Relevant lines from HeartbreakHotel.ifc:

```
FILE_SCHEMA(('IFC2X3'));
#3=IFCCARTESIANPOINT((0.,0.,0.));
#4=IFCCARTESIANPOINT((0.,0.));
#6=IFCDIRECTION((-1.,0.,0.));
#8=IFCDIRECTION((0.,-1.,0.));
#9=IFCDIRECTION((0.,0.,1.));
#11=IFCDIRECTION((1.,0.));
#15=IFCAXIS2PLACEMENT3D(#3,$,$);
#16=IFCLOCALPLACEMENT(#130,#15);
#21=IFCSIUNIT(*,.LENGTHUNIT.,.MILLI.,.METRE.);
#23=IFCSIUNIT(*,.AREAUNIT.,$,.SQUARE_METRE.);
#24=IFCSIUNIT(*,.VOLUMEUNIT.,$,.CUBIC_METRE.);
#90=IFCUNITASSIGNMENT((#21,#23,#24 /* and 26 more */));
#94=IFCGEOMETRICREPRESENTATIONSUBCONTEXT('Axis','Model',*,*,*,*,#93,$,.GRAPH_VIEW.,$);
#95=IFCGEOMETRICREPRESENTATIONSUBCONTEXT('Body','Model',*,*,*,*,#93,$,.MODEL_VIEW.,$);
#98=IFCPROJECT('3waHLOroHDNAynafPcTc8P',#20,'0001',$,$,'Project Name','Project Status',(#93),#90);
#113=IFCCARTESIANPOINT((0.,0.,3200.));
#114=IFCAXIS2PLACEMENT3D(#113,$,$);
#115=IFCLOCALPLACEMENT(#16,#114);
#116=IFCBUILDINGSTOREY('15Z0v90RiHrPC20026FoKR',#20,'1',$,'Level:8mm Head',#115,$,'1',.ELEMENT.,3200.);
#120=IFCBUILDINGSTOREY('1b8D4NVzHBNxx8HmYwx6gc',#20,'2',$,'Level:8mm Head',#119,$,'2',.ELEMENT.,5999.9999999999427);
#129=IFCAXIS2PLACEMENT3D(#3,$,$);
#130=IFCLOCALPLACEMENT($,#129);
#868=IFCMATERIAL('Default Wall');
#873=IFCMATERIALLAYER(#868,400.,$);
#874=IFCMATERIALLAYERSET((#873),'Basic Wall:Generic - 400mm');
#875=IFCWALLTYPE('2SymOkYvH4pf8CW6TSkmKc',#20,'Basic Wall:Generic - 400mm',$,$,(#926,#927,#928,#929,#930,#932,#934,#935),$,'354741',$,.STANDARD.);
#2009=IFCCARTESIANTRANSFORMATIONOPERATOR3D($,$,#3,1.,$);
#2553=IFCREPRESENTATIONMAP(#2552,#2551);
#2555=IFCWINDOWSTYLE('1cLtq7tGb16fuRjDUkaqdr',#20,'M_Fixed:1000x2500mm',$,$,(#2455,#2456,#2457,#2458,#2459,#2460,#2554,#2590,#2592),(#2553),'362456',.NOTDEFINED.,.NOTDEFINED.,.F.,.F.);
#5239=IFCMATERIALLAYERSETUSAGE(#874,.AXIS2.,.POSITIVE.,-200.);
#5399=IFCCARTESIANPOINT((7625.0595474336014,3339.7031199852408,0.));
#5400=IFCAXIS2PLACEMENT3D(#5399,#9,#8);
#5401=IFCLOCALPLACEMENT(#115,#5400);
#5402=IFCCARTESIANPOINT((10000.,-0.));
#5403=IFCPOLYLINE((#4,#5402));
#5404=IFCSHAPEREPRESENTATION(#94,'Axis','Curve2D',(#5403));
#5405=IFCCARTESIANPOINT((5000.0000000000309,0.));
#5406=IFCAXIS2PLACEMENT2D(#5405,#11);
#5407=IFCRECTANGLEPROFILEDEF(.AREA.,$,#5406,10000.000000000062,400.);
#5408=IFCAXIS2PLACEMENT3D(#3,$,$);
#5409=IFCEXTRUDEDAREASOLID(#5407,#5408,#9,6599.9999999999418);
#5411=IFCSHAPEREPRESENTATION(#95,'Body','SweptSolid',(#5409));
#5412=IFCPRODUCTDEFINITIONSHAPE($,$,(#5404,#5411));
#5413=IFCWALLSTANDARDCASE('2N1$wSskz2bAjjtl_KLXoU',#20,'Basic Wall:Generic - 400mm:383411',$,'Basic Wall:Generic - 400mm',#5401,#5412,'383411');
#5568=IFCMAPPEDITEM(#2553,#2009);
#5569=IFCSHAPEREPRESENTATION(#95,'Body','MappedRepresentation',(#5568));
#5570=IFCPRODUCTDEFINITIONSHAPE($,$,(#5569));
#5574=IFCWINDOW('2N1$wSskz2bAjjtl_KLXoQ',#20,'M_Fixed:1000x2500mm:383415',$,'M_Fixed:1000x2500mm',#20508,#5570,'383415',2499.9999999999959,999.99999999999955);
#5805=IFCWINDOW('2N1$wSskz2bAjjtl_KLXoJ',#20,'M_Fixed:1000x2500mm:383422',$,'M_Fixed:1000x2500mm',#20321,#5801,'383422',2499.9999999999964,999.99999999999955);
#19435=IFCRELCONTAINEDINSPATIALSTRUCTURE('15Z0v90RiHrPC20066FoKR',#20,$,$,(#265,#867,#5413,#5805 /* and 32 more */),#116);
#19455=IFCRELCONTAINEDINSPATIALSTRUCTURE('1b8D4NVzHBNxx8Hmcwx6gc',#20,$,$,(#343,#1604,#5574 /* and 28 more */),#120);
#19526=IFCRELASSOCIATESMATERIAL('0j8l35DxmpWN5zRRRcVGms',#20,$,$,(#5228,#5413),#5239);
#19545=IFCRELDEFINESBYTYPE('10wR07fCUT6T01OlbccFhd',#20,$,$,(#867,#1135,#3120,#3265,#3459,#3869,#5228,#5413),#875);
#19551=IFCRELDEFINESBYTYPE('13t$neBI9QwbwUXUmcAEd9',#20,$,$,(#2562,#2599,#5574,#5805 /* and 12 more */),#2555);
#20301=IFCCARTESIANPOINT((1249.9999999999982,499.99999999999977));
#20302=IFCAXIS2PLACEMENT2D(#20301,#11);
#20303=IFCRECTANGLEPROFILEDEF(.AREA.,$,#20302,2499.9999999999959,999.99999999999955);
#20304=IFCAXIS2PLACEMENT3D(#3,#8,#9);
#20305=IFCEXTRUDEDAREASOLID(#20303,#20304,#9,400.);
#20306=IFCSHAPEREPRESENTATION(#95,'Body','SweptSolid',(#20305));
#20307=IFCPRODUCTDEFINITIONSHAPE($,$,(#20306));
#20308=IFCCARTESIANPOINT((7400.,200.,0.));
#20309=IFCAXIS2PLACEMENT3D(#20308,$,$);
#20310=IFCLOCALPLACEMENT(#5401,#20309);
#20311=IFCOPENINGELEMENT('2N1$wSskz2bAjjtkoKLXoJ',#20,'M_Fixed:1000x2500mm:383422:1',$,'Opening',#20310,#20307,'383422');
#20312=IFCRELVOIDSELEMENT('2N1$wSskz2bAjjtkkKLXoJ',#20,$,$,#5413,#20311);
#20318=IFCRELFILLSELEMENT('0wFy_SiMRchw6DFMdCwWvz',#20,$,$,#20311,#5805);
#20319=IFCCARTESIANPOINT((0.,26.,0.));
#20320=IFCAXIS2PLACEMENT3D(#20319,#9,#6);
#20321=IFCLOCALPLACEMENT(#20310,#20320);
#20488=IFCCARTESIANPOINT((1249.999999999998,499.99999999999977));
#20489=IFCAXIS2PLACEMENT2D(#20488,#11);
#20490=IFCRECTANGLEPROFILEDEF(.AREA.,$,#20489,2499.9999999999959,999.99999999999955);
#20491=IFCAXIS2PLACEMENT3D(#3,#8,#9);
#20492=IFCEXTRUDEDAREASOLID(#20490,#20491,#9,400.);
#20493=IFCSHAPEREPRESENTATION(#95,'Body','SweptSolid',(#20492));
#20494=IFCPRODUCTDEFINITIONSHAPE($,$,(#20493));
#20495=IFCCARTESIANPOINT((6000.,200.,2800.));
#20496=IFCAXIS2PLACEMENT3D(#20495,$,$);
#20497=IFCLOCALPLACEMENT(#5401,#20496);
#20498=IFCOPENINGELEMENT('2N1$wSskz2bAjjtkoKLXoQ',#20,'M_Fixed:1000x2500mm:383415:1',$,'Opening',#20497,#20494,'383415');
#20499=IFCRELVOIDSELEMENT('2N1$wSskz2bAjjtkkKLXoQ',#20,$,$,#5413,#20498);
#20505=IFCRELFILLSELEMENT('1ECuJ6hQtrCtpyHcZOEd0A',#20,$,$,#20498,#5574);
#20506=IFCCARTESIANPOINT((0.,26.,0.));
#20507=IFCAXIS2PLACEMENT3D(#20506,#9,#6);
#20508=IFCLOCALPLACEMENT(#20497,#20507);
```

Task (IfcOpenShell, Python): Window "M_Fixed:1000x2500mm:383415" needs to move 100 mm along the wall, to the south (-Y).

```python
import ifcopenshell
import ifcopenshell.api.geometry
import ifcopenshell.util.placement

model = ifcopenshell.open("HeartbreakHotel.ifc")

window = model.by_id(5574)
opening = window.FillsVoids[0].RelatingOpeningElement
wall = opening.VoidsElements[0].RelatingBuildingElement

wall_matrix = ifcopenshell.util.placement.get_local_placement(wall.ObjectPlacement)
shift = wall_matrix[:3, 0] * 100.0
before = ifcopenshell.util.placement.get_local_placement(window.ObjectPlacement)[:3, 3].copy()

# The window is placed relative to its opening, so it follows when the opening moves.
matrix = ifcopenshell.util.placement.get_local_placement(opening.ObjectPlacement)
matrix[:3, 3] += shift
ifcopenshell.api.geometry.edit_object_placement(
    model, product=opening, matrix=matrix, is_si=False, should_transform_children=True
)

after = ifcopenshell.util.placement.get_local_placement(window.ObjectPlacement)[:3, 3]
print("window moved by", (after - before).round(3) + 0.0)

model.write("HeartbreakHotel_edited.ifc")
```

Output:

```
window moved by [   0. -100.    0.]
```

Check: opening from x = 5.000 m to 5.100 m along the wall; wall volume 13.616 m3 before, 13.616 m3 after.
